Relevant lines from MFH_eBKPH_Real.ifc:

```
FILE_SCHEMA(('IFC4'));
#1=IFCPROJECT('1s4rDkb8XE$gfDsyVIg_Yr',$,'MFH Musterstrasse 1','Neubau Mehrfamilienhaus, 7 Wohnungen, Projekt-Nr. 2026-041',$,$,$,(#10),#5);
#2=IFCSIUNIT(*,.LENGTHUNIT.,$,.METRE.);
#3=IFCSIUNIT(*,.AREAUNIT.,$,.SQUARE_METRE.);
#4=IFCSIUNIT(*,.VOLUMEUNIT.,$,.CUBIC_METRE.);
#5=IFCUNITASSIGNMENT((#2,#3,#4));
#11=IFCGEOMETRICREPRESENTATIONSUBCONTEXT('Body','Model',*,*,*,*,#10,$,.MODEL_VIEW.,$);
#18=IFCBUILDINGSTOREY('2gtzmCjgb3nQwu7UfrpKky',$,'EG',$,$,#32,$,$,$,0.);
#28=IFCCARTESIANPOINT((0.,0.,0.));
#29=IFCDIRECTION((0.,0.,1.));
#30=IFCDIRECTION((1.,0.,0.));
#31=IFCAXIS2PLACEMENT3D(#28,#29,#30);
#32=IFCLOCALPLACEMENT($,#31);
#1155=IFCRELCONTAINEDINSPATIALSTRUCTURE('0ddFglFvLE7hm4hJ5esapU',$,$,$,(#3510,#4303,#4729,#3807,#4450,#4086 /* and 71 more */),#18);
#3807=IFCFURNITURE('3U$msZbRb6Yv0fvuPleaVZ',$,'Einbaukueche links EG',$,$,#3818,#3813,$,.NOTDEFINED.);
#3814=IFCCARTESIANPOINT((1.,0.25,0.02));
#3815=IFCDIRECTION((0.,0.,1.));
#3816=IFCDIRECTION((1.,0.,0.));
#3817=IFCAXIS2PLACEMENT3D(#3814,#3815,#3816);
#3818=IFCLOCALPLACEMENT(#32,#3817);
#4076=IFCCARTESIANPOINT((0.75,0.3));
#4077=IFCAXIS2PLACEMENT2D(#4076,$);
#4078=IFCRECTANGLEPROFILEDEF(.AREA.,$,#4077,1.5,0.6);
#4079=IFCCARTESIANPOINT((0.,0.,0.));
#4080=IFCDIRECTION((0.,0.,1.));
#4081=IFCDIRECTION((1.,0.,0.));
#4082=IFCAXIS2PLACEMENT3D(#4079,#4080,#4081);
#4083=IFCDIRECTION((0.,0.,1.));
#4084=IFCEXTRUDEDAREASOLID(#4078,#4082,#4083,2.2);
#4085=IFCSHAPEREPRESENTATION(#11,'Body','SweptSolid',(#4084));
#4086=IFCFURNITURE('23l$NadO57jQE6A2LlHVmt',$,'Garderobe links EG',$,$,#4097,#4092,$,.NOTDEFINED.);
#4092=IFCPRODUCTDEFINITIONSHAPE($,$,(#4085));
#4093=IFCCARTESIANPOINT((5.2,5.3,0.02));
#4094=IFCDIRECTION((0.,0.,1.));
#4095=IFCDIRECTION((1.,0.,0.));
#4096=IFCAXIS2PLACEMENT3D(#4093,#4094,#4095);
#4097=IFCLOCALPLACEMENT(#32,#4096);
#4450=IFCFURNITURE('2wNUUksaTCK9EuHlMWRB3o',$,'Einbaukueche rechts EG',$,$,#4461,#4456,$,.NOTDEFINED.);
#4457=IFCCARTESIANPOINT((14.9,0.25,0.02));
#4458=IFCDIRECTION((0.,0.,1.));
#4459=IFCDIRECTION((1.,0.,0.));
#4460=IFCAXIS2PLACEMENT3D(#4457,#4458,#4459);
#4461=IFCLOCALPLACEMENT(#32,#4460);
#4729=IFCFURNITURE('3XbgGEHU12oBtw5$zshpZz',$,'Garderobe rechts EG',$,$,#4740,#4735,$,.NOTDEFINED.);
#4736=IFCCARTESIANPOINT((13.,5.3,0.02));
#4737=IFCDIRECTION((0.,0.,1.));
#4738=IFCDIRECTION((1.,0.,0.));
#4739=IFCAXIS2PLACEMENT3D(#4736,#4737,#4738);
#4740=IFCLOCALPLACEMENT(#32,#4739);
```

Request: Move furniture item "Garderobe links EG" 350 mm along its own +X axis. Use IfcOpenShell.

```python
import ifcopenshell
import ifcopenshell.api.geometry
import ifcopenshell.util.placement
import ifcopenshell.util.unit

model = ifcopenshell.open("MFH_eBKPH_Real.ifc")
unit_scale = ifcopenshell.util.unit.calculate_unit_scale(model)

item = model.by_guid("23l$NadO57jQE6A2LlHVmt")
matrix = ifcopenshell.util.placement.get_local_placement(item.ObjectPlacement)
matrix[:3, 3] += matrix[:3, 0] * 0.35 / unit_scale
ifcopenshell.api.geometry.edit_object_placement(model, product=item, matrix=matrix, is_si=False)

print(ifcopenshell.util.placement.get_local_placement(item.ObjectPlacement).round(3) + 0.0)

model.write("MFH_eBKPH_Real_edited.ifc")
```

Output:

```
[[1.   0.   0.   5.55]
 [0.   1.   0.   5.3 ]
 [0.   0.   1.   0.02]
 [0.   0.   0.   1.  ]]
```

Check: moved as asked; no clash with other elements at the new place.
